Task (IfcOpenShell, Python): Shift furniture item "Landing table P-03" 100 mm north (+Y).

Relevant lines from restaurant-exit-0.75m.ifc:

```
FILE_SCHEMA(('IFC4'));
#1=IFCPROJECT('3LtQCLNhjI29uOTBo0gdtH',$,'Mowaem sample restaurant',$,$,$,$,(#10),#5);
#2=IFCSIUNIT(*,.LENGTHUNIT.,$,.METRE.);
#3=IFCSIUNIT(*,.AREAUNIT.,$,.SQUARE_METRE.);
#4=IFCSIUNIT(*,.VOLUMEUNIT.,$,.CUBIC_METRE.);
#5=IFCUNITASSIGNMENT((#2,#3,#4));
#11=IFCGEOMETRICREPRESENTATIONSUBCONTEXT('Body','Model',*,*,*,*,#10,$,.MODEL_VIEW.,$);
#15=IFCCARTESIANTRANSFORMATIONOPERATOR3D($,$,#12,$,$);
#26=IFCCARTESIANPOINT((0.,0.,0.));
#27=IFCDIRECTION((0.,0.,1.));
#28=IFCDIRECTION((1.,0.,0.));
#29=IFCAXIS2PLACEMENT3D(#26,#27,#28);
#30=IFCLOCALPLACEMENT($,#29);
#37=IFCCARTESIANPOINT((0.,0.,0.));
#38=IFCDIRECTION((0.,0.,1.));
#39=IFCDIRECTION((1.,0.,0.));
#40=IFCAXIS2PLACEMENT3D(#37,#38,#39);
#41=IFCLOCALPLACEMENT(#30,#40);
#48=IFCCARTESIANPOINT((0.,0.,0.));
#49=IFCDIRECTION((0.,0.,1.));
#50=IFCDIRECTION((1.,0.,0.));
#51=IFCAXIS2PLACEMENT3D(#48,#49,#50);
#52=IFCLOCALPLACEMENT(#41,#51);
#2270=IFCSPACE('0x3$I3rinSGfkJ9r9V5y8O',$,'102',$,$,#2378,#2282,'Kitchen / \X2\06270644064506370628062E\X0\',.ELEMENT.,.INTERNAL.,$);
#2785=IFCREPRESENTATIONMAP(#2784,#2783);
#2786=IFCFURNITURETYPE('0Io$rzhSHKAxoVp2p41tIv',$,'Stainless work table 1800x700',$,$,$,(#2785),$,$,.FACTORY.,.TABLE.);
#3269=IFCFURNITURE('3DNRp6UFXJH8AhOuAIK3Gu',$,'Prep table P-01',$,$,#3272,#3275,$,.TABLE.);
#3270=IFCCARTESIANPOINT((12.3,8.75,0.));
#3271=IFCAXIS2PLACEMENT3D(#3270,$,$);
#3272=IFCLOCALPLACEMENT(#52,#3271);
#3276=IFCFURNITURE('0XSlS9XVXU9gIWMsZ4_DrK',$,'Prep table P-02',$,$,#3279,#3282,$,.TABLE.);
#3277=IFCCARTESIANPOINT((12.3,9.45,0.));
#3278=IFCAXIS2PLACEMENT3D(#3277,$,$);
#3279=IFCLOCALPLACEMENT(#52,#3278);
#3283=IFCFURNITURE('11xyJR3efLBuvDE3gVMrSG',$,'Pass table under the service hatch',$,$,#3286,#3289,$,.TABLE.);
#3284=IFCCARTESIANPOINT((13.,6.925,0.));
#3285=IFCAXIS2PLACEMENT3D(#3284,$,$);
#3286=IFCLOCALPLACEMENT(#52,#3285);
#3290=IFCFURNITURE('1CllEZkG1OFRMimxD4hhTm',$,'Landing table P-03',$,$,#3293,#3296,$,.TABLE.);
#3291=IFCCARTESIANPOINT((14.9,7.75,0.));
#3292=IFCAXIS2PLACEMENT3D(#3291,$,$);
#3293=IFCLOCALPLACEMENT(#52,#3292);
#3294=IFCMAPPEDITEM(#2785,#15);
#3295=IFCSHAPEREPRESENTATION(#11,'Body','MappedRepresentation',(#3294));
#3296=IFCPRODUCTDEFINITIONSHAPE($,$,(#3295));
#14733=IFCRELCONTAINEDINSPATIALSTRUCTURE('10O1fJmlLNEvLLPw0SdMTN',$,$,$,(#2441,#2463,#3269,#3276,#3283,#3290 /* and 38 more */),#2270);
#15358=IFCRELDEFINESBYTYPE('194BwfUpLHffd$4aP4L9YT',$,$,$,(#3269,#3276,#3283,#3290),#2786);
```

```python
import ifcopenshell
import ifcopenshell.api.geometry
import ifcopenshell.util.placement

model = ifcopenshell.open("restaurant-exit-0.75m.ifc")

item = model.by_id(3290)
matrix = ifcopenshell.util.placement.get_local_placement(item.ObjectPlacement)
matrix[1, 3] += 0.1
ifcopenshell.api.geometry.edit_object_placement(model, product=item, matrix=matrix, is_si=False)

print(ifcopenshell.util.placement.get_local_placement(item.ObjectPlacement).round(3) + 0.0)

model.write("restaurant-exit-0.75m_v2.ifc")
```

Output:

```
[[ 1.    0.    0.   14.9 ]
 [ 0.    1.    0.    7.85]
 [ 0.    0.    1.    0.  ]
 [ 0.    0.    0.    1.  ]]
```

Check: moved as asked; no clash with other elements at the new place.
